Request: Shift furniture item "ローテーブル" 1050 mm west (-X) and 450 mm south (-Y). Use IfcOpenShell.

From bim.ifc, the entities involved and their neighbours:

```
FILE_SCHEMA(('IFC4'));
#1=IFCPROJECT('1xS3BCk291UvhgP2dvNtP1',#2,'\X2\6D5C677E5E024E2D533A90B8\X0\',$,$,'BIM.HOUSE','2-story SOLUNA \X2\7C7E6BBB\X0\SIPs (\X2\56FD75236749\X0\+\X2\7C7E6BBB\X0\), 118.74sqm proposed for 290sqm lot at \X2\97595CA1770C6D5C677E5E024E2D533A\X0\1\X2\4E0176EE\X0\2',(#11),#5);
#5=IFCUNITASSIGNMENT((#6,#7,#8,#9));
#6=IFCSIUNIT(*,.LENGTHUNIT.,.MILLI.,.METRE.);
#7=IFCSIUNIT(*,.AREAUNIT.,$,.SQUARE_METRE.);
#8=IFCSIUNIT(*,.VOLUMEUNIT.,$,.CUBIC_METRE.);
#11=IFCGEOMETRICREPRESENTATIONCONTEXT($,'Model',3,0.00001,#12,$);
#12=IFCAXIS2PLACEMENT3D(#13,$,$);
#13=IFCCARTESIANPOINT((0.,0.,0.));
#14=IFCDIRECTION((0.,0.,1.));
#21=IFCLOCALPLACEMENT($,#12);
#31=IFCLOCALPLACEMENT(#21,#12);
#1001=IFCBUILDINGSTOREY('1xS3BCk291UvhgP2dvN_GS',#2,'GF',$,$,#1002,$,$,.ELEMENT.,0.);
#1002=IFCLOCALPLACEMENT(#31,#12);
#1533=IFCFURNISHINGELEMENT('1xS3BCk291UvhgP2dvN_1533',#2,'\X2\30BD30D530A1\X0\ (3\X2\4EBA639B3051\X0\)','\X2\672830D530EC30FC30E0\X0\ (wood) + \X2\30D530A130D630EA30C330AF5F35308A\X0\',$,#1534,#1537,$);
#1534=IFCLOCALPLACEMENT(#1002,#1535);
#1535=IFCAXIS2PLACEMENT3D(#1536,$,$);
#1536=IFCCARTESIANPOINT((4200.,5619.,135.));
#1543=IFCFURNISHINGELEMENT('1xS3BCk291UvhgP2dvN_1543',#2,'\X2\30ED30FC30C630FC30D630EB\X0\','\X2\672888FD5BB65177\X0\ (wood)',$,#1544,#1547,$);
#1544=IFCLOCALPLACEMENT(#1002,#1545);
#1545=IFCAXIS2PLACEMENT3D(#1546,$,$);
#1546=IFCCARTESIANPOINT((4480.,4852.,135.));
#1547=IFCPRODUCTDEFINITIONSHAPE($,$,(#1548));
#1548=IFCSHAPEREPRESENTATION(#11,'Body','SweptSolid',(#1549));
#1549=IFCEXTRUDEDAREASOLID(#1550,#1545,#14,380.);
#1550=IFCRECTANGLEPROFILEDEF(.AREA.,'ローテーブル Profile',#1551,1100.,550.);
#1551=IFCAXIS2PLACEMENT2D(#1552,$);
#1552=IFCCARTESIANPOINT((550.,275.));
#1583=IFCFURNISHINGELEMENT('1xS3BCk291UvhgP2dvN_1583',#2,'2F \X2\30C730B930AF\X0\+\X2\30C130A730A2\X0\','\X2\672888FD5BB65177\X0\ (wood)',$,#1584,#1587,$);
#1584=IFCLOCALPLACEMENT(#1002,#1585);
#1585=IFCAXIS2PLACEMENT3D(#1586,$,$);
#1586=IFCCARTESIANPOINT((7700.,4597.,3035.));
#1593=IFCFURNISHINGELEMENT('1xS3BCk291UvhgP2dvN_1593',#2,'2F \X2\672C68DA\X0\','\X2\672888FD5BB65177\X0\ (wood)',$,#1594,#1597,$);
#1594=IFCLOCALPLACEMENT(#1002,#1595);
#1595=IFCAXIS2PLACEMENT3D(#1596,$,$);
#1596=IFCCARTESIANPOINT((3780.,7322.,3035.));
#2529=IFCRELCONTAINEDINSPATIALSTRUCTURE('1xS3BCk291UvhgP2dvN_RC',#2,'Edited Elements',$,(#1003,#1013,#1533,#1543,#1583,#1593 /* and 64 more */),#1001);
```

```python
import ifcopenshell
import ifcopenshell.api.geometry
import ifcopenshell.util.placement
import ifcopenshell.util.unit

model = ifcopenshell.open("bim.ifc")
unit_scale = ifcopenshell.util.unit.calculate_unit_scale(model)

item = model.by_id(1543)
matrix = ifcopenshell.util.placement.get_local_placement(item.ObjectPlacement)
matrix[0, 3] -= 1.05 / unit_scale
matrix[1, 3] -= 0.45 / unit_scale
ifcopenshell.api.geometry.edit_object_placement(model, product=item, matrix=matrix, is_si=False)

print(ifcopenshell.util.placement.get_local_placement(item.ObjectPlacement).round(3) + 0.0)

model.write("bim_v2.ifc")
```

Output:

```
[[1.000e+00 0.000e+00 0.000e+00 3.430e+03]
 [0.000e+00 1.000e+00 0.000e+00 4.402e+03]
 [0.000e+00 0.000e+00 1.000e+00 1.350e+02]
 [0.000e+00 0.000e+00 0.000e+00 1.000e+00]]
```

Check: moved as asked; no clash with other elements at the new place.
